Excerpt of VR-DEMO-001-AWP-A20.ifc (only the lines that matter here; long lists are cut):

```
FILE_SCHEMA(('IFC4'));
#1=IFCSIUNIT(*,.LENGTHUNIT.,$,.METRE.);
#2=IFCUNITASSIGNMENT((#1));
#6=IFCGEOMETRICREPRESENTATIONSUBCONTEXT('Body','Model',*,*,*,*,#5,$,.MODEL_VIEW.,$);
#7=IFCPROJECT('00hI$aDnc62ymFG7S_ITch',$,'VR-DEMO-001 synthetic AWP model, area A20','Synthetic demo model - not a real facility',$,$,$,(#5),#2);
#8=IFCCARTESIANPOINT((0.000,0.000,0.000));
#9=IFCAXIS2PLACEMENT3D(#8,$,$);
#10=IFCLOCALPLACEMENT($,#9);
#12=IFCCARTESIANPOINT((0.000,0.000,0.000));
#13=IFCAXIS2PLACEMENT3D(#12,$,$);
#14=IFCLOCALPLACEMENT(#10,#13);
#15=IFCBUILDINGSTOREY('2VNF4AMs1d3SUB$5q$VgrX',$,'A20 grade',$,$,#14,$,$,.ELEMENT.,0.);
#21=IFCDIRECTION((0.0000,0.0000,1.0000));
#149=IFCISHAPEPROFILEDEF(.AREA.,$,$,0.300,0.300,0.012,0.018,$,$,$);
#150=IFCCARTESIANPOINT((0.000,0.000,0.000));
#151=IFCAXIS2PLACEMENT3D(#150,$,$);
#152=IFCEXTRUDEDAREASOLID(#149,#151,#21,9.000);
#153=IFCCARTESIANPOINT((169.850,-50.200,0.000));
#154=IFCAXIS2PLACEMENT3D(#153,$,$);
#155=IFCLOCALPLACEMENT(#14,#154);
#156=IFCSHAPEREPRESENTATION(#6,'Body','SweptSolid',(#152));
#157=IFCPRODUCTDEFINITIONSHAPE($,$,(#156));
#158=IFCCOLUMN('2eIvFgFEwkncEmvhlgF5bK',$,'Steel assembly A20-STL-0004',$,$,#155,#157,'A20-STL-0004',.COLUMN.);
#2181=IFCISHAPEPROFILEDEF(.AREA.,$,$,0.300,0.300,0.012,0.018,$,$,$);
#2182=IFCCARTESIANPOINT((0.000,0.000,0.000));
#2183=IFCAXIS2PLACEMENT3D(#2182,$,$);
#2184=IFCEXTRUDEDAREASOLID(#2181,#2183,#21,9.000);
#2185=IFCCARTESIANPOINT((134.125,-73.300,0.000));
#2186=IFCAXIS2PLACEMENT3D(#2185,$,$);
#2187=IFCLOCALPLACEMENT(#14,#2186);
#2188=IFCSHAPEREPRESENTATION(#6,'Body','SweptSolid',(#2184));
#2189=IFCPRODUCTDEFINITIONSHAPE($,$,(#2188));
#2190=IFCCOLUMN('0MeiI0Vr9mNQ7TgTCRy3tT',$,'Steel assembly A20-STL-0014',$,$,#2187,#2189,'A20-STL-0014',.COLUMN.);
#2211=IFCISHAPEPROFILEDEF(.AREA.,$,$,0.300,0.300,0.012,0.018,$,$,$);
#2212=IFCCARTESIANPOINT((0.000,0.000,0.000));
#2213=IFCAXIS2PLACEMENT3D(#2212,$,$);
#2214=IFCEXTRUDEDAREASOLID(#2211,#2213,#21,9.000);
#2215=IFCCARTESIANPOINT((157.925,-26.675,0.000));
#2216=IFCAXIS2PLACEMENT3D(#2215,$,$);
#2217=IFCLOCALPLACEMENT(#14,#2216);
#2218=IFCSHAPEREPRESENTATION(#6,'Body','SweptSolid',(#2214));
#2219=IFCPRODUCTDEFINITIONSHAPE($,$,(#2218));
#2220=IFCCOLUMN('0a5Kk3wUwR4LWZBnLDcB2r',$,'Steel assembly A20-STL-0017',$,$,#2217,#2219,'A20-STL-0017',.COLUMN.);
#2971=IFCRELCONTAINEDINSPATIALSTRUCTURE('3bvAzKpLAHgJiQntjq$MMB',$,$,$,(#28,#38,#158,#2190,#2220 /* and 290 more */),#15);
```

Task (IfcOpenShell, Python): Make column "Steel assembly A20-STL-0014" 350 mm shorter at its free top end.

```python
import ifcopenshell
import ifcopenshell.util.representation

model = ifcopenshell.open("VR-DEMO-001-AWP-A20.ifc")

member = model.by_guid("0MeiI0Vr9mNQ7TgTCRy3tT")
change = -0.35

# The extrusion runs towards the end named, so only its depth changes.
body = ifcopenshell.util.representation.get_representation(member, "Model", "Body")
solid = body.Items[0]
old_length = solid.Depth
solid.Depth += change

print(f"length {old_length:g} -> {solid.Depth:g}")

model.write("VR-DEMO-001-AWP-A20_v2.ifc")
```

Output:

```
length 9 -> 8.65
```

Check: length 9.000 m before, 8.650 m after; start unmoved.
